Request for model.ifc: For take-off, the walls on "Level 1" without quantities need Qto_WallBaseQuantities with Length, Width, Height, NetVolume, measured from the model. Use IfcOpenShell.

First a look at what the model holds.

```python
import ifcopenshell
import ifcopenshell.util.element
import ifcopenshell.util.unit

model = ifcopenshell.open("model.ifc")
print(model.schema)
for unit_type in ("LENGTHUNIT", "AREAUNIT", "VOLUMEUNIT"):
    print(unit_type, ifcopenshell.util.unit.calculate_unit_scale(model, unit_type))
storey = next(s for s in model.by_type("IfcBuildingStorey") if s.Name == "Level 1")
walls = [e for e in ifcopenshell.util.element.get_decomposition(storey) if e.is_a("IfcWall")]
for e in sorted(walls, key=lambda e: e.id()):
    print(e.id(), e.is_a(), e.Name, list(ifcopenshell.util.element.get_psets(e, qtos_only=True)), sep=" | ")
```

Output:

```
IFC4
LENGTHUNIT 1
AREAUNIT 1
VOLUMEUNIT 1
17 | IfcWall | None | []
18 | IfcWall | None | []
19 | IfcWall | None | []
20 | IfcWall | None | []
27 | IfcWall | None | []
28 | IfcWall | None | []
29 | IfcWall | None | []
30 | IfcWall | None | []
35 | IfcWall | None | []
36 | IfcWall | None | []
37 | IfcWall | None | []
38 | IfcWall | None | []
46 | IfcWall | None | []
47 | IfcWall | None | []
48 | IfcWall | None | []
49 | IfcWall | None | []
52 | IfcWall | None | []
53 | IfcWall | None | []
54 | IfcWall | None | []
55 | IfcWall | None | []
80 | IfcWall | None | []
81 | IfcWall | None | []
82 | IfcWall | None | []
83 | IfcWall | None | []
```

```python
import ifcopenshell
import ifcopenshell.api.pset
import ifcopenshell.geom
import ifcopenshell.util.element
import ifcopenshell.util.shape
import ifcopenshell.util.unit

model = ifcopenshell.open("model.ifc")
unit_scale = ifcopenshell.util.unit.calculate_unit_scale(model)
volume_scale = ifcopenshell.util.unit.calculate_unit_scale(model, "VOLUMEUNIT")
settings = ifcopenshell.geom.settings()

storey = next(s for s in model.by_type("IfcBuildingStorey") if s.Name == "Level 1")
walls = [e for e in ifcopenshell.util.element.get_decomposition(storey) if e.is_a("IfcWall")]

for e in sorted(walls, key=lambda e: e.id()):
    if ifcopenshell.util.element.get_psets(e, qtos_only=True, should_inherit=False):
        continue
    # Geometry comes back in metres, in the element's own axes.
    shape = ifcopenshell.geom.create_shape(settings, e)
    values = {
        "Length": ifcopenshell.util.shape.get_x(shape.geometry) / unit_scale,
        "Width": ifcopenshell.util.shape.get_y(shape.geometry) / unit_scale,
        "Height": ifcopenshell.util.shape.get_z(shape.geometry) / unit_scale,
        "NetVolume": ifcopenshell.util.shape.get_volume(shape.geometry) / volume_scale,
    }
    qto = ifcopenshell.api.pset.add_qto(model, product=e, name="Qto_WallBaseQuantities")
    ifcopenshell.api.pset.edit_qto(model, qto=qto, properties=values)
    print(e.id(), {k: round(v, 3) for k, v in values.items()})

model.write("model_edited.ifc")
```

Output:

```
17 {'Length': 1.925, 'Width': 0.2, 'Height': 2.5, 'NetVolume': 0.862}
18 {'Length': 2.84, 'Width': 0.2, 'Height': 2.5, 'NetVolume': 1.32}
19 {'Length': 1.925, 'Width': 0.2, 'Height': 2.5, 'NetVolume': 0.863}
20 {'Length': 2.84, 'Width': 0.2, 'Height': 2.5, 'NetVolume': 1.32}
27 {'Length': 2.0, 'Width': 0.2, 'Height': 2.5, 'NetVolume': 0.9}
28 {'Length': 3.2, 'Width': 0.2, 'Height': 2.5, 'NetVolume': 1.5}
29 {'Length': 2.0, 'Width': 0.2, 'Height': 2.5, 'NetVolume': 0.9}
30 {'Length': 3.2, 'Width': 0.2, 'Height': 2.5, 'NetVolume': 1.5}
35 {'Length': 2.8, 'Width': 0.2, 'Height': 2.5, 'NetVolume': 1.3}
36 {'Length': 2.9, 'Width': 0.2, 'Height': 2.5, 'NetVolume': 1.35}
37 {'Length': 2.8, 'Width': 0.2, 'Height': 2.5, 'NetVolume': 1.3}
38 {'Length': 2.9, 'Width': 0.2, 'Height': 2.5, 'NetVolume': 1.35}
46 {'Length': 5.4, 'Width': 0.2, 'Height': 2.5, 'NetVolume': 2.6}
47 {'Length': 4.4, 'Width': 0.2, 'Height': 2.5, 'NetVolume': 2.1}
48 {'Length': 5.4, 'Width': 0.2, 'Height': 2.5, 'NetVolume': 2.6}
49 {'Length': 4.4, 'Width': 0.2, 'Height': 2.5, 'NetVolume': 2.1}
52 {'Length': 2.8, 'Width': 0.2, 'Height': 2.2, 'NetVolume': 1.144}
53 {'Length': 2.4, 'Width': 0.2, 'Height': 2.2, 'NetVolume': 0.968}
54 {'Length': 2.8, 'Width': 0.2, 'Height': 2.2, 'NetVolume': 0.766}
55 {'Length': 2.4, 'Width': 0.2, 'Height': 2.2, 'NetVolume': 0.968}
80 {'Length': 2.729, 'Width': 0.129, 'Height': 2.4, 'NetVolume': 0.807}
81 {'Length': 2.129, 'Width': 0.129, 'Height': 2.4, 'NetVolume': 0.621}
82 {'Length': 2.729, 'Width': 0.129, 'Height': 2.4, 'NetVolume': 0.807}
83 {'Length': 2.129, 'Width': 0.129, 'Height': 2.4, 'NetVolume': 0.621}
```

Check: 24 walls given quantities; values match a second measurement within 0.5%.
